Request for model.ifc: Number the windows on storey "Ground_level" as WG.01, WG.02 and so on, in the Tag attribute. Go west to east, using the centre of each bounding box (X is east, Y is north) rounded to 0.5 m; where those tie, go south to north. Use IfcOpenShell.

First a look at what the model holds.

```python
import ifcopenshell
import ifcopenshell.util.element
import ifcopenshell.util.placement

model = ifcopenshell.open("model.ifc")
print(model.schema)
storey = next(s for s in model.by_type("IfcBuildingStorey") if s.Name == "Ground_level")
windows = [e for e in ifcopenshell.util.element.get_decomposition(storey) if e.is_a("IfcWindow")]
for e in sorted(windows, key=lambda e: e.id()):
    origin = ifcopenshell.util.placement.get_local_placement(e.ObjectPlacement)[:3, 3]
    print(e.id(), e.Tag, e.Name, origin.round(2) + 0.0, sep=" | ")
```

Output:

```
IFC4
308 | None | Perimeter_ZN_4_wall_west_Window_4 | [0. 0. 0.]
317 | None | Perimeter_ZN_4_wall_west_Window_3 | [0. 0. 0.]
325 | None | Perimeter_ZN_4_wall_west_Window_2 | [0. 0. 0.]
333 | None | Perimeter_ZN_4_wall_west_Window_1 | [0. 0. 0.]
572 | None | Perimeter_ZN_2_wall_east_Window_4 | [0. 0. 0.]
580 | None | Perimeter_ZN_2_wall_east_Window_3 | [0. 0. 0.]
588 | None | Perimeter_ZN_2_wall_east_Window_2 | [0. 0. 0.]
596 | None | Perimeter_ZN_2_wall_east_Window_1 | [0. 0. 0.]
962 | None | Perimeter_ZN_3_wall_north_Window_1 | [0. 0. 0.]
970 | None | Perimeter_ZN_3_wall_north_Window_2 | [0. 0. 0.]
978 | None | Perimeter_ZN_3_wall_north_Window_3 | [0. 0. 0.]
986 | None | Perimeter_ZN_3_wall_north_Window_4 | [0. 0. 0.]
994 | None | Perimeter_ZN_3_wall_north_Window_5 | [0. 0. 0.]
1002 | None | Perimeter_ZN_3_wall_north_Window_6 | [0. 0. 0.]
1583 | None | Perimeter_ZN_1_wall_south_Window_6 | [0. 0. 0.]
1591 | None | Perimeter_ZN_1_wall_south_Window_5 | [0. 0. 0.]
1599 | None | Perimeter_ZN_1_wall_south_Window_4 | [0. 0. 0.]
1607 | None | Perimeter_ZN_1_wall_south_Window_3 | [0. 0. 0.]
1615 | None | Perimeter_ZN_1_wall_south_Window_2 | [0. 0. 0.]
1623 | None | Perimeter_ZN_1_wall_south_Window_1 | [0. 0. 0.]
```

```python
import ifcopenshell
import ifcopenshell.geom
import ifcopenshell.util.element
import ifcopenshell.util.shape

model = ifcopenshell.open("model.ifc")
settings = ifcopenshell.geom.settings()
settings.set("use-world-coords", True)


def centre(element):
    shape = ifcopenshell.geom.create_shape(settings, element)
    return ifcopenshell.util.shape.get_bbox_centroid(shape.geometry)


storey = next(s for s in model.by_type("IfcBuildingStorey") if s.Name == "Ground_level")
windows = [e for e in ifcopenshell.util.element.get_decomposition(storey) if e.is_a("IfcWindow")]

# Insertion points can sit at a corner or the storey origin, so sort by the geometry (in metres).
centres = {e: centre(e) for e in windows}
windows.sort(key=lambda e: (round(centres[e][0] / 0.5), centres[e][1]))

for i, e in enumerate(windows, start=1):
    number = f"WG.{i:02d}"
    e.Tag = number
    print(e.id(), number)

model.write("model_updated.ifc")
```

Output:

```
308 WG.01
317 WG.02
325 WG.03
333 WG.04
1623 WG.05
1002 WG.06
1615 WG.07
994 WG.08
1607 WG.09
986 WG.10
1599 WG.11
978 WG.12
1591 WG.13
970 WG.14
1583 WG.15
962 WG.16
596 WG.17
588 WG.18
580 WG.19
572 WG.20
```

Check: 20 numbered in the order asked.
